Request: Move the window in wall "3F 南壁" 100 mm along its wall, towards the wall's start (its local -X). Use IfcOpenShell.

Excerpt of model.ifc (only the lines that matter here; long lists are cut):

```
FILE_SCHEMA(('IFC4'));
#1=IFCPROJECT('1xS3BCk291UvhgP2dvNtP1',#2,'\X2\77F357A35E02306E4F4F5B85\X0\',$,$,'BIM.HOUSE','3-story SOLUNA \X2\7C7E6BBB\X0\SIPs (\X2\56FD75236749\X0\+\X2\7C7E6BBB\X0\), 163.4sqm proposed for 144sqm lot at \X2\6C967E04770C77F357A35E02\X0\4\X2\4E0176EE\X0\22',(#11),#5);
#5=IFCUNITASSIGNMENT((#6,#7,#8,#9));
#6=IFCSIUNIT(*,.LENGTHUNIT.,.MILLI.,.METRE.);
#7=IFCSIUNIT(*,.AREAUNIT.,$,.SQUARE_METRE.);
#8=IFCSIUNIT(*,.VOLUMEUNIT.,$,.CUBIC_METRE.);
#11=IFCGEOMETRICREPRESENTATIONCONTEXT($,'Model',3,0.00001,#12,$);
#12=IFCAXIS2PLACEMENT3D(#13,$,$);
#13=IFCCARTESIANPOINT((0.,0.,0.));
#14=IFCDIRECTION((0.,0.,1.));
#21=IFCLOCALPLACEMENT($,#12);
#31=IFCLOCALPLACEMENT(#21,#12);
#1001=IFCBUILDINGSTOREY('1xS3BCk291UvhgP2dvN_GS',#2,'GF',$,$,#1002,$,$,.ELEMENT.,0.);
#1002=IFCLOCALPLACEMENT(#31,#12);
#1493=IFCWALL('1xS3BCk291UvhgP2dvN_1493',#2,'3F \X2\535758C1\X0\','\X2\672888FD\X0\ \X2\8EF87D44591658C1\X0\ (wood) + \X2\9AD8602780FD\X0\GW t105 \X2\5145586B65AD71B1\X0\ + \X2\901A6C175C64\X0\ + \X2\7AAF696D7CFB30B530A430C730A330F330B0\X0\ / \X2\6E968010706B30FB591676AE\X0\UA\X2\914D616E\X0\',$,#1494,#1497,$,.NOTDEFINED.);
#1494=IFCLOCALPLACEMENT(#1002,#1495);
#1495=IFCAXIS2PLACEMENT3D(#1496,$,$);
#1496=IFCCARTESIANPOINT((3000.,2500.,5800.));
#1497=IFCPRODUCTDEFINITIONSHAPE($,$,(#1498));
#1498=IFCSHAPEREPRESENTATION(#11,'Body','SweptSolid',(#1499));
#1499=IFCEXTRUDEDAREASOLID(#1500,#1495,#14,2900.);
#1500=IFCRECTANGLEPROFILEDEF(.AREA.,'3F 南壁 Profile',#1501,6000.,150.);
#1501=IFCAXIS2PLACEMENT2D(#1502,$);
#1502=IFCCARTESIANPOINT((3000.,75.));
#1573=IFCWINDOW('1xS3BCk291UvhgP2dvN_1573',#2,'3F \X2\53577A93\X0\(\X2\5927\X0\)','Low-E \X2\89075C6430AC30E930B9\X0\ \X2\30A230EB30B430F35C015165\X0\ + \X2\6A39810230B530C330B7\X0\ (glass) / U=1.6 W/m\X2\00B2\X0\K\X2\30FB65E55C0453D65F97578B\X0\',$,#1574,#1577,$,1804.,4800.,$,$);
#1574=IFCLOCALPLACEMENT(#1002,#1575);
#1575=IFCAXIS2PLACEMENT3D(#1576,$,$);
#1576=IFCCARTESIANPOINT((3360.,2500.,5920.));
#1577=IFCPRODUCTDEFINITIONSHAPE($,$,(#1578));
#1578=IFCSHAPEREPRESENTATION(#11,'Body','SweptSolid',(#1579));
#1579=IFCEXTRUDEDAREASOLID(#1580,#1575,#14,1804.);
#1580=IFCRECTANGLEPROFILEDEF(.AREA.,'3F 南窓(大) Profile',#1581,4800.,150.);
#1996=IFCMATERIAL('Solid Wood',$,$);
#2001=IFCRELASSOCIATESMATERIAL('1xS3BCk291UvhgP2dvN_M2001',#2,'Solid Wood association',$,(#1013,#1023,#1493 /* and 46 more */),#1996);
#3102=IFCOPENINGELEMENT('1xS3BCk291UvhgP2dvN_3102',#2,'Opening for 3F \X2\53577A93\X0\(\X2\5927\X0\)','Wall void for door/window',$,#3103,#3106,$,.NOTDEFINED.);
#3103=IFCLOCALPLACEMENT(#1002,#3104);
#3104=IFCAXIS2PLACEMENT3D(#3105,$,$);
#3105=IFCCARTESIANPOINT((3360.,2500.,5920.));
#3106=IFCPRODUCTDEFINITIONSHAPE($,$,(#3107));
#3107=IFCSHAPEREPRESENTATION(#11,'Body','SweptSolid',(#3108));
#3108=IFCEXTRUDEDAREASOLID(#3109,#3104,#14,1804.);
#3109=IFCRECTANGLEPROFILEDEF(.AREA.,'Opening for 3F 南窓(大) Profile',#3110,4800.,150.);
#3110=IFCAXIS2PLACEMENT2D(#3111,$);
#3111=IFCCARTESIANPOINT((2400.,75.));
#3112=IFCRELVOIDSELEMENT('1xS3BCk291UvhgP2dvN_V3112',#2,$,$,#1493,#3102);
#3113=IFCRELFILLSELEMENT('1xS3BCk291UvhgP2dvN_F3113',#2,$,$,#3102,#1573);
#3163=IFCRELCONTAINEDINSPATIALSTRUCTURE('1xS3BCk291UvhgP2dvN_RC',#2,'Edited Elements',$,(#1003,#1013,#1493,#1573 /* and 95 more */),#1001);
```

```python
import ifcopenshell
import ifcopenshell.api.geometry
import ifcopenshell.util.placement
import ifcopenshell.util.unit

model = ifcopenshell.open("model.ifc")
unit_scale = ifcopenshell.util.unit.calculate_unit_scale(model)

window = model.by_id(1573)
opening = window.FillsVoids[0].RelatingOpeningElement
wall = opening.VoidsElements[0].RelatingBuildingElement

wall_matrix = ifcopenshell.util.placement.get_local_placement(wall.ObjectPlacement)
shift = wall_matrix[:3, 0] * -0.1 / unit_scale
before = ifcopenshell.util.placement.get_local_placement(window.ObjectPlacement)[:3, 3].copy()

# The window is not placed relative to its opening, so move both.
for product in (opening, window):
    matrix = ifcopenshell.util.placement.get_local_placement(product.ObjectPlacement)
    matrix[:3, 3] += shift
    ifcopenshell.api.geometry.edit_object_placement(model, product=product, matrix=matrix, is_si=False)

after = ifcopenshell.util.placement.get_local_placement(window.ObjectPlacement)[:3, 3]
print("window moved by", (after - before).round(3) + 0.0)

model.write("model_rev.ifc")
```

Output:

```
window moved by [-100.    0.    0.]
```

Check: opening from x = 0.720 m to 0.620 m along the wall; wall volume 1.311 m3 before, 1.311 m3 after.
